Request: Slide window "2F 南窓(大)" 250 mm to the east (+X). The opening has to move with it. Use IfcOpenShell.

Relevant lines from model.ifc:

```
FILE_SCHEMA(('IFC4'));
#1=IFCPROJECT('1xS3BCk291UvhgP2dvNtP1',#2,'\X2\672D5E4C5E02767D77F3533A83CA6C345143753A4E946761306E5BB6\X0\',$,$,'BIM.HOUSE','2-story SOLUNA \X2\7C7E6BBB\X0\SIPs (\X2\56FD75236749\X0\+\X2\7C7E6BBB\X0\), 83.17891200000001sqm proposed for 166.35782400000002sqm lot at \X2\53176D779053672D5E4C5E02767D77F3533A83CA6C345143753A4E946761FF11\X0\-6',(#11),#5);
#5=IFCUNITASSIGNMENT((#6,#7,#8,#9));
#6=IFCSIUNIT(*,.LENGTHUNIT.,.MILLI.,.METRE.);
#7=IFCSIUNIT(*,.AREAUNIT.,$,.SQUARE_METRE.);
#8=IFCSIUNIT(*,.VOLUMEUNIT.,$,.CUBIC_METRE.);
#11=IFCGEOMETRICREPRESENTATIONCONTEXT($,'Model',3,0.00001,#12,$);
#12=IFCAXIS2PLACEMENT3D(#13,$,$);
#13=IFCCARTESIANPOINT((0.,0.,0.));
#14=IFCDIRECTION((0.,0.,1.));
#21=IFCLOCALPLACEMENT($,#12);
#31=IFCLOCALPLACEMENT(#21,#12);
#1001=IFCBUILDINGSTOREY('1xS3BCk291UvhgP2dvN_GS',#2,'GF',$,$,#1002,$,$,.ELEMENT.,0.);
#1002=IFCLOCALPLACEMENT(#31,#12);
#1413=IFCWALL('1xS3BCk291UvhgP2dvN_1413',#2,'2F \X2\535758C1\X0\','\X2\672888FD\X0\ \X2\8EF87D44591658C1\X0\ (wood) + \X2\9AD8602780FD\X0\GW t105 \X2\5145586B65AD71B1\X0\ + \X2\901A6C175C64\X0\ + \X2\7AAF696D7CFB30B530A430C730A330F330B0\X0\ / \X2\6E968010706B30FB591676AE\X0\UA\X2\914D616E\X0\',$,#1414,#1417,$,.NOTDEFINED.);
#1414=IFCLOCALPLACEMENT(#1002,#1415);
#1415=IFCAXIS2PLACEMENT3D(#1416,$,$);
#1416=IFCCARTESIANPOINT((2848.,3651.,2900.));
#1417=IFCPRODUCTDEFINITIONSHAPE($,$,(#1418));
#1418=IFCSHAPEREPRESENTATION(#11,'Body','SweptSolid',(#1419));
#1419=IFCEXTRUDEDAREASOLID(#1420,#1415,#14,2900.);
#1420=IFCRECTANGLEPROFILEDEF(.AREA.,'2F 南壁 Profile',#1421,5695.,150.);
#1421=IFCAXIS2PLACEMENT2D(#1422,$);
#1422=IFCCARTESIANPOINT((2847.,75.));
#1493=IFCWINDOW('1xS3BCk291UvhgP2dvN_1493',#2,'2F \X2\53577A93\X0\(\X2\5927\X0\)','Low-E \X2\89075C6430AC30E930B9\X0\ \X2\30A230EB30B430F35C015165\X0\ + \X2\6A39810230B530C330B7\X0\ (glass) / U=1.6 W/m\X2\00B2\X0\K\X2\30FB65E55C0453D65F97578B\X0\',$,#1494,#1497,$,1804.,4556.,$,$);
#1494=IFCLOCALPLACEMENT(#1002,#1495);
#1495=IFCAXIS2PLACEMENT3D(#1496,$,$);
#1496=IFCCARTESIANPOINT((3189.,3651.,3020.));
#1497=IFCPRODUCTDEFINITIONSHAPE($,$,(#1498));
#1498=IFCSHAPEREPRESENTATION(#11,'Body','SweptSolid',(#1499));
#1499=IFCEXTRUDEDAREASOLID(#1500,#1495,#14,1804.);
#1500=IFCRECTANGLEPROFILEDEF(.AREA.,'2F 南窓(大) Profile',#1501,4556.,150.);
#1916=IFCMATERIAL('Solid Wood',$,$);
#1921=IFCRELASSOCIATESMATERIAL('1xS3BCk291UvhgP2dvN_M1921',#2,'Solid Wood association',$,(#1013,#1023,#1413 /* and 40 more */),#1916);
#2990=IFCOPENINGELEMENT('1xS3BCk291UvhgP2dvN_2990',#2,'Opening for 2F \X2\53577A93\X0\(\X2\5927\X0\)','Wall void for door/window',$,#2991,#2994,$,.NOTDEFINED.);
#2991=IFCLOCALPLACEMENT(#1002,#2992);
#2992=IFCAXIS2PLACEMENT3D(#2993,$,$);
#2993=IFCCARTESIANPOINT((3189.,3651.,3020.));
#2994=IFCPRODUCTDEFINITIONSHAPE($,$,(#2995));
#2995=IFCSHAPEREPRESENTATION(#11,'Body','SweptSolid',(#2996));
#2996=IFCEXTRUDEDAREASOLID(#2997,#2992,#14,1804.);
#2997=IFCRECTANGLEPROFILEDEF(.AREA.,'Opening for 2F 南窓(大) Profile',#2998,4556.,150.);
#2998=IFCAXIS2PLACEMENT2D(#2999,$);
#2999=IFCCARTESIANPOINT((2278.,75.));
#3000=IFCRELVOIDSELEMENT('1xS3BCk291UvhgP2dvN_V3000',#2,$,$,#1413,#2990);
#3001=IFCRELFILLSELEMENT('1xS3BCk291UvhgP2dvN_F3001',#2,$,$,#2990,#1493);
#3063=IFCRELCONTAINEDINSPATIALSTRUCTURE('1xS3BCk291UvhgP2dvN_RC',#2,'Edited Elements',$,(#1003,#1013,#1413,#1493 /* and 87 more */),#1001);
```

```python
import ifcopenshell
import ifcopenshell.api.geometry
import ifcopenshell.util.placement
import ifcopenshell.util.unit

model = ifcopenshell.open("model.ifc")
unit_scale = ifcopenshell.util.unit.calculate_unit_scale(model)

window = model.by_guid("1xS3BCk291UvhgP2dvN_1493")
opening = window.FillsVoids[0].RelatingOpeningElement
wall = opening.VoidsElements[0].RelatingBuildingElement

wall_matrix = ifcopenshell.util.placement.get_local_placement(wall.ObjectPlacement)
shift = wall_matrix[:3, 0] * 0.25 / unit_scale
before = ifcopenshell.util.placement.get_local_placement(window.ObjectPlacement)[:3, 3].copy()

# The window is not placed relative to its opening, so move both.
for product in (opening, window):
    matrix = ifcopenshell.util.placement.get_local_placement(product.ObjectPlacement)
    matrix[:3, 3] += shift
    ifcopenshell.api.geometry.edit_object_placement(model, product=product, matrix=matrix, is_si=False)

after = ifcopenshell.util.placement.get_local_placement(window.ObjectPlacement)[:3, 3]
print("window moved by", (after - before).round(3) + 0.0)

model.write("model_rev.ifc")
```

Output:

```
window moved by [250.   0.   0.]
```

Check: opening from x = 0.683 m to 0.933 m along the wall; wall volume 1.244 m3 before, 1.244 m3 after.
